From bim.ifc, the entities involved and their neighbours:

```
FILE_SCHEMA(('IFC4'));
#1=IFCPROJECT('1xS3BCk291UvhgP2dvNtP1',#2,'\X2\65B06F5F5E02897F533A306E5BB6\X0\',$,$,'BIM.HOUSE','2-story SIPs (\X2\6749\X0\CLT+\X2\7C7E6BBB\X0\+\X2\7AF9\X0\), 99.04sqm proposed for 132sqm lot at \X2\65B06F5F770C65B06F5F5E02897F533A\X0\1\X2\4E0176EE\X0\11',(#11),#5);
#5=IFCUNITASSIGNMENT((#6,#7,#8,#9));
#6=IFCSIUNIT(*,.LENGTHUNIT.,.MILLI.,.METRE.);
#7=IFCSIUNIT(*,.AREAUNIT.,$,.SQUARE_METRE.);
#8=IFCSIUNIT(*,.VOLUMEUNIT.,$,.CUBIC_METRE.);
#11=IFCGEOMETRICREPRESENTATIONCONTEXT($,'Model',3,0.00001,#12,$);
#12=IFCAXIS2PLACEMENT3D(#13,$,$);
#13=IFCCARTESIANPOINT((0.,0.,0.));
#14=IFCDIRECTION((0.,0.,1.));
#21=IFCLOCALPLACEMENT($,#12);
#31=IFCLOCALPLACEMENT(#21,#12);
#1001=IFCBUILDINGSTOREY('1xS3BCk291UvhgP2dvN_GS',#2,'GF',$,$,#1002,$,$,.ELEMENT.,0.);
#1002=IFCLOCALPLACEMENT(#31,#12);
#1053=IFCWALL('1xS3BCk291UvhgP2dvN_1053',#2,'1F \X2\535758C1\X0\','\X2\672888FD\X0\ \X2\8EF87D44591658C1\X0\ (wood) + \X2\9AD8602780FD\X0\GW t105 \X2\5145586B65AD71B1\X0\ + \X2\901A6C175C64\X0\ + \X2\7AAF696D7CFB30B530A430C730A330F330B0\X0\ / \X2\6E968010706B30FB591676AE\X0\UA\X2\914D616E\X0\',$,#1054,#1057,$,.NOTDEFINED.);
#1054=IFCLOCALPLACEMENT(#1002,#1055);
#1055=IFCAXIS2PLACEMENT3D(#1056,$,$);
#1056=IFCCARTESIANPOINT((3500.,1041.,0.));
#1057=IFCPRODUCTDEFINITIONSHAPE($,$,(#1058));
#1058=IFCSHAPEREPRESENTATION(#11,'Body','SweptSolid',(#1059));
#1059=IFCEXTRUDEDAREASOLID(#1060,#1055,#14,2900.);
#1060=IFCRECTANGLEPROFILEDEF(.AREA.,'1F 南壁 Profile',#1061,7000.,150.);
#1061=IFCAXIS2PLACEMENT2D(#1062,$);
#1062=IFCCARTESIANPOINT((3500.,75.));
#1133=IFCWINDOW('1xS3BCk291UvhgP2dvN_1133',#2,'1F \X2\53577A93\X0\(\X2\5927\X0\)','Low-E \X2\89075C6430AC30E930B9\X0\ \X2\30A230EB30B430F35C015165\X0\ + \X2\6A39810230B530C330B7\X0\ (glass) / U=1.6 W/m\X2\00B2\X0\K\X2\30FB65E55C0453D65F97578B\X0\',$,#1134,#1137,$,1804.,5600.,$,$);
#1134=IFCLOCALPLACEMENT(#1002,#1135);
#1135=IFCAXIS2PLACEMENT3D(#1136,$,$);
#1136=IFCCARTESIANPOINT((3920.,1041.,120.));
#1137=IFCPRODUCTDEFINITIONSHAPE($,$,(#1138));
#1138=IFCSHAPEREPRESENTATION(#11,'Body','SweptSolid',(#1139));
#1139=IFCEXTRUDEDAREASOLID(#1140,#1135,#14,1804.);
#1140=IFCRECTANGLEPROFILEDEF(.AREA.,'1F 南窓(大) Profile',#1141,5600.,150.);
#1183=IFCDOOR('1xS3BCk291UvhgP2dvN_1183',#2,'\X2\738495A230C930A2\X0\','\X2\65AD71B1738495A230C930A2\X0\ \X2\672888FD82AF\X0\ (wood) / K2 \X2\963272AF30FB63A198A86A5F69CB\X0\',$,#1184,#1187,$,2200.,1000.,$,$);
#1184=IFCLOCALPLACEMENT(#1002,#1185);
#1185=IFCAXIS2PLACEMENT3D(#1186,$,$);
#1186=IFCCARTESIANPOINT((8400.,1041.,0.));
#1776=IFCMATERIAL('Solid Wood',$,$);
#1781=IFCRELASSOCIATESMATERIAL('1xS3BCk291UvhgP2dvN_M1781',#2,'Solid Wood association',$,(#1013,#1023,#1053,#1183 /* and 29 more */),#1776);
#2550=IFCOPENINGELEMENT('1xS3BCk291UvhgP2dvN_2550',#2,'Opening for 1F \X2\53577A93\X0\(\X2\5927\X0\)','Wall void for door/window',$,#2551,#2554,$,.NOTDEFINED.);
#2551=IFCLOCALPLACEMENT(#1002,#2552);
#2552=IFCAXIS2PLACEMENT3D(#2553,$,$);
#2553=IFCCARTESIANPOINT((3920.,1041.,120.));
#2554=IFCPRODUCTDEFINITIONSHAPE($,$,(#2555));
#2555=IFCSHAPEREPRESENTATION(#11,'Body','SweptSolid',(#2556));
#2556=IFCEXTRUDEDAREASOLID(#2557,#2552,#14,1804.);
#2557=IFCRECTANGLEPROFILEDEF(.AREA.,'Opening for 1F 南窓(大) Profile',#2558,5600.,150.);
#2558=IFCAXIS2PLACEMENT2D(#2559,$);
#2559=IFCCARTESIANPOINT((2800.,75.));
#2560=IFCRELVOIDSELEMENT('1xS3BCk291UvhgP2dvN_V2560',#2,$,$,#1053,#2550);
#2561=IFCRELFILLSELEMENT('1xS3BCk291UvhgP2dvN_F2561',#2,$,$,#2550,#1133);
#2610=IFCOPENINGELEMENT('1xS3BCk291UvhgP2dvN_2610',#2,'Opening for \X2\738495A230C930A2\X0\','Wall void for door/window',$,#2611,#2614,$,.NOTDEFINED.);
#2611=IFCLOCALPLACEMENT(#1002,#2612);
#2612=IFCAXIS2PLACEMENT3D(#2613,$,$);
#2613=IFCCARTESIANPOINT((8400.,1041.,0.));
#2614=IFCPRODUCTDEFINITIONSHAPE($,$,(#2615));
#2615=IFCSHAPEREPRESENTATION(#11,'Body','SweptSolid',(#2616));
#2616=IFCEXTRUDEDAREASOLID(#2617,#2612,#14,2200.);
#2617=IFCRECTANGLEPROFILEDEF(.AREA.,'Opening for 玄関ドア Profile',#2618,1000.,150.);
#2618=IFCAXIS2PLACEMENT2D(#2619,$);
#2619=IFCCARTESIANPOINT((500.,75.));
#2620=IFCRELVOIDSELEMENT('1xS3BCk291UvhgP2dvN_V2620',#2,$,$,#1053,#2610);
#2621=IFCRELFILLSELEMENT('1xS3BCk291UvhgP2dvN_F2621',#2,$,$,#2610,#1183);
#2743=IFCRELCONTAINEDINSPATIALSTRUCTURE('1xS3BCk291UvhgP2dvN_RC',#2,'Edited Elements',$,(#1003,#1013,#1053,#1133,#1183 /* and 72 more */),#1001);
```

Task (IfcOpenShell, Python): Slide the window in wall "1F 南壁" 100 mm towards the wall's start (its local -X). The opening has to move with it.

```python
import ifcopenshell
import ifcopenshell.api.geometry
import ifcopenshell.util.placement
import ifcopenshell.util.unit

model = ifcopenshell.open("bim.ifc")
unit_scale = ifcopenshell.util.unit.calculate_unit_scale(model)

window = model.by_id(1133)
opening = window.FillsVoids[0].RelatingOpeningElement
wall = opening.VoidsElements[0].RelatingBuildingElement

wall_matrix = ifcopenshell.util.placement.get_local_placement(wall.ObjectPlacement)
shift = wall_matrix[:3, 0] * -0.1 / unit_scale
before = ifcopenshell.util.placement.get_local_placement(window.ObjectPlacement)[:3, 3].copy()

# The window is not placed relative to its opening, so move both.
for product in (opening, window):
    matrix = ifcopenshell.util.placement.get_local_placement(product.ObjectPlacement)
    matrix[:3, 3] += shift
    ifcopenshell.api.geometry.edit_object_placement(model, product=product, matrix=matrix, is_si=False)

after = ifcopenshell.util.placement.get_local_placement(window.ObjectPlacement)[:3, 3]
print("window moved by", (after - before).round(3) + 0.0)

model.write("bim-out.ifc")
```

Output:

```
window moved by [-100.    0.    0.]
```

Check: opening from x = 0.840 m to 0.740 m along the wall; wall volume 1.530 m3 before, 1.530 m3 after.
